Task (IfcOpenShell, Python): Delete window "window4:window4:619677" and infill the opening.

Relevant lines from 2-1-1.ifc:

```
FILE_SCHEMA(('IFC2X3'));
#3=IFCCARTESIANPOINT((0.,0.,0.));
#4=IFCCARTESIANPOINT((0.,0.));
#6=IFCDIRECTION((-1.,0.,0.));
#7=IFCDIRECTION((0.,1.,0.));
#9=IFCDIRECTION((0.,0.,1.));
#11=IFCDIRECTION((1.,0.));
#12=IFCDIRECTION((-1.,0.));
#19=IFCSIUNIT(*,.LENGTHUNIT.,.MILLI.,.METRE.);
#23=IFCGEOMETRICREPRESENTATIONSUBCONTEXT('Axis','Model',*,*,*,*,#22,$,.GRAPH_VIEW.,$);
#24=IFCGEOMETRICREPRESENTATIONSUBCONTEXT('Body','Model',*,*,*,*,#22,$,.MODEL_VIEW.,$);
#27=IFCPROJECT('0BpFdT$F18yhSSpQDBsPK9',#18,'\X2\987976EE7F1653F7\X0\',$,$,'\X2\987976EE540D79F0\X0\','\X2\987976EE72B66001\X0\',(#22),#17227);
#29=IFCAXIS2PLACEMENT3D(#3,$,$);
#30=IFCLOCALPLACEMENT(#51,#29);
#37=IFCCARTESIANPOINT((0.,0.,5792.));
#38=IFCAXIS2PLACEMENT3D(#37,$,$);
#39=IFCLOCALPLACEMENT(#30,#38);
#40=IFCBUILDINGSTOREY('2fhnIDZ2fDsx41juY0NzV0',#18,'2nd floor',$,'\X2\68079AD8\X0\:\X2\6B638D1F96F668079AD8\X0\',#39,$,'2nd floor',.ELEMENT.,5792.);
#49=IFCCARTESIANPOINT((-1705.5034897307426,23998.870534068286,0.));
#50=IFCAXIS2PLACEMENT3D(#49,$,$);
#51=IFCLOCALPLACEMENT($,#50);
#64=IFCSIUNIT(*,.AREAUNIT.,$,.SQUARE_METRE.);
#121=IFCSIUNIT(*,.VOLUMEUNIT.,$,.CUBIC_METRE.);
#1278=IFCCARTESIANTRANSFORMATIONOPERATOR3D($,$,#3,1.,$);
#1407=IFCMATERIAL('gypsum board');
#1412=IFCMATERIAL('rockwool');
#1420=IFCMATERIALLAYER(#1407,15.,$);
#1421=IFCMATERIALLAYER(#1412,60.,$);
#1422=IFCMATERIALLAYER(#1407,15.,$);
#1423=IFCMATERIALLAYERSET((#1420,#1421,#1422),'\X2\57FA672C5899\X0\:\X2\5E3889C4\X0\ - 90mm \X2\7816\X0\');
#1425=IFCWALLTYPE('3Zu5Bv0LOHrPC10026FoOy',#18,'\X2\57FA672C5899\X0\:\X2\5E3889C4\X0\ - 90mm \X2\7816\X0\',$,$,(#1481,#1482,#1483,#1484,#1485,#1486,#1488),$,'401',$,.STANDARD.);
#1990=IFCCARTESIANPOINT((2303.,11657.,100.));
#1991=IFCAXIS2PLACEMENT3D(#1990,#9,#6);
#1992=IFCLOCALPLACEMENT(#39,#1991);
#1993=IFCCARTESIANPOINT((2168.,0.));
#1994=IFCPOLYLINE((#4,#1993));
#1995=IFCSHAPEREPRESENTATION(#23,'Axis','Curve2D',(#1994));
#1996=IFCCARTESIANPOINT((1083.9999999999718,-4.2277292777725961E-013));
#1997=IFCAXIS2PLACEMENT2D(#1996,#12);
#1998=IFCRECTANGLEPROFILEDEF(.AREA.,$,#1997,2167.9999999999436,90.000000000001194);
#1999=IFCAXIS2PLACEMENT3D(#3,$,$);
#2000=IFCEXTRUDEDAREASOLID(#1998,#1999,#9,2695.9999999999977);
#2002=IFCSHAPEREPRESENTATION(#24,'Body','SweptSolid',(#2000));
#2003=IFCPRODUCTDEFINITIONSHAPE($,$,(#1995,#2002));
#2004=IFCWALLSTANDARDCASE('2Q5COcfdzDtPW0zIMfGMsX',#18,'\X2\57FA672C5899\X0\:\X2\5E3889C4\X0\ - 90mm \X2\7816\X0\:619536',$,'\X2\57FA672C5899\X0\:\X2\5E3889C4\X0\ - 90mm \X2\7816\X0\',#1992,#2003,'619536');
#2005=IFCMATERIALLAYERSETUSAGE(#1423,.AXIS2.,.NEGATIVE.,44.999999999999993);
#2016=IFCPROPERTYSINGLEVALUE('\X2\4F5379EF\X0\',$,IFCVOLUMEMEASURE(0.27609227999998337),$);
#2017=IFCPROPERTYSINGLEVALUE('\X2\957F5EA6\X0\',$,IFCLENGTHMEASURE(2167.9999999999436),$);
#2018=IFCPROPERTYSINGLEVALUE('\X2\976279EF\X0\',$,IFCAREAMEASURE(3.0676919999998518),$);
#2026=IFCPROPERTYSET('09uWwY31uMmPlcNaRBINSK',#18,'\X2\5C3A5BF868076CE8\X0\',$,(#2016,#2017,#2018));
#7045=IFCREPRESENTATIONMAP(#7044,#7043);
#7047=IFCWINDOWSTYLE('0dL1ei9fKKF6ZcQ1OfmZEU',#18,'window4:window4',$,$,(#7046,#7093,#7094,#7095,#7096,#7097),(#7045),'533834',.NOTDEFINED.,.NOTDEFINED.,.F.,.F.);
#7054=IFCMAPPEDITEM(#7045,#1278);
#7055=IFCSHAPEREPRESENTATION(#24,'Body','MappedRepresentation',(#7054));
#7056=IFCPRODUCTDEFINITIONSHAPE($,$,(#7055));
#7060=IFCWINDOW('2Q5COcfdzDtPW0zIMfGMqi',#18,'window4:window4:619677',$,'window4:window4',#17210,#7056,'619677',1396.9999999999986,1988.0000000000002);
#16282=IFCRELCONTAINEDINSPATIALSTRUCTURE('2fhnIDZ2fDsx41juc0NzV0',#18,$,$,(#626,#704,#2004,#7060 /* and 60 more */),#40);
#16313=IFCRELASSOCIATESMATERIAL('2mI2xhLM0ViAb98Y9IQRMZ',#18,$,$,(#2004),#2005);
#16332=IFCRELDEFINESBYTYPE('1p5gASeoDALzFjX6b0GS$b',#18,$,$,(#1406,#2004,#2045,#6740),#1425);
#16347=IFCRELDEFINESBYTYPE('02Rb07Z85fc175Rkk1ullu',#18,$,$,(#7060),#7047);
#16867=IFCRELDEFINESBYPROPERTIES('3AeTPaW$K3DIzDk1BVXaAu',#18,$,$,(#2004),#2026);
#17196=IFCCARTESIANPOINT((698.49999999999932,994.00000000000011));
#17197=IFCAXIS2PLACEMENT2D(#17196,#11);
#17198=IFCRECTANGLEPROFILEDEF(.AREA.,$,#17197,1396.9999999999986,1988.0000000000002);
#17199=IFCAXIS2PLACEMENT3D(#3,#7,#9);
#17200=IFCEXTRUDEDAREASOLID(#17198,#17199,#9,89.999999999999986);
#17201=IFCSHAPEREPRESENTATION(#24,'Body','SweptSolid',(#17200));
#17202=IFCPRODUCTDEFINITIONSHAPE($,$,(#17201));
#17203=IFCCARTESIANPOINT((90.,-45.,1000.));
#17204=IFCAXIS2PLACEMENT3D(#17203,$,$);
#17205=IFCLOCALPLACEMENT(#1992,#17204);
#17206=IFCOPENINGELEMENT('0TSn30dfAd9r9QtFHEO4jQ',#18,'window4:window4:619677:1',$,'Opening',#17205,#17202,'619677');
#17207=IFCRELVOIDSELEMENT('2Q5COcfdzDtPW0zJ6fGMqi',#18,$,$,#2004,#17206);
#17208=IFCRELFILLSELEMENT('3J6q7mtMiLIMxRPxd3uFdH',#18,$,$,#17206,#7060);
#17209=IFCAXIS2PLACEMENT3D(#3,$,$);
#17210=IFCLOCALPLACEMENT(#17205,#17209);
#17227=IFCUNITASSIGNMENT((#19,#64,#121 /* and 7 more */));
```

```python
import ifcopenshell
import ifcopenshell.api.feature
import ifcopenshell.api.pset
import ifcopenshell.api.root
import ifcopenshell.geom
import ifcopenshell.util.element
import ifcopenshell.util.shape
import ifcopenshell.util.unit

model = ifcopenshell.open("2-1-1.ifc")
area_scale = ifcopenshell.util.unit.calculate_unit_scale(model, "AREAUNIT")
volume_scale = ifcopenshell.util.unit.calculate_unit_scale(model, "VOLUMEUNIT")
settings = ifcopenshell.geom.settings()


def volume(element):
    """Net volume in cubic metres, openings subtracted."""
    shape = ifcopenshell.geom.create_shape(settings, element)
    return ifcopenshell.util.shape.get_volume(shape.geometry)


window = model.by_guid("2Q5COcfdzDtPW0zIMfGMqi")
opening = window.FillsVoids[0].RelatingOpeningElement
wall = opening.VoidsElements[0].RelatingBuildingElement
before = volume(wall)

ifcopenshell.api.root.remove_product(model, product=window)
ifcopenshell.api.feature.remove_feature(model, feature=opening)

after = volume(wall)
thickness = 0.09  # wall thickness in metres

# Update the wall's stored quantities.
pset = model.by_id(ifcopenshell.util.element.get_pset(wall, "尺寸标注", should_inherit=False)["id"])
ifcopenshell.api.pset.edit_pset(model, pset=pset, properties={
    "体积": model.create_entity("IfcVolumeMeasure", after / volume_scale),
    "面积": model.create_entity("IfcAreaMeasure", after / thickness / area_scale),
})

print(f"wall volume {before:.3f} -> {after:.3f} m3")

model.write("2-1-1_rev.ifc")
```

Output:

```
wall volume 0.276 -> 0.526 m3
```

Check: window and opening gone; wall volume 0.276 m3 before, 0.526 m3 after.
